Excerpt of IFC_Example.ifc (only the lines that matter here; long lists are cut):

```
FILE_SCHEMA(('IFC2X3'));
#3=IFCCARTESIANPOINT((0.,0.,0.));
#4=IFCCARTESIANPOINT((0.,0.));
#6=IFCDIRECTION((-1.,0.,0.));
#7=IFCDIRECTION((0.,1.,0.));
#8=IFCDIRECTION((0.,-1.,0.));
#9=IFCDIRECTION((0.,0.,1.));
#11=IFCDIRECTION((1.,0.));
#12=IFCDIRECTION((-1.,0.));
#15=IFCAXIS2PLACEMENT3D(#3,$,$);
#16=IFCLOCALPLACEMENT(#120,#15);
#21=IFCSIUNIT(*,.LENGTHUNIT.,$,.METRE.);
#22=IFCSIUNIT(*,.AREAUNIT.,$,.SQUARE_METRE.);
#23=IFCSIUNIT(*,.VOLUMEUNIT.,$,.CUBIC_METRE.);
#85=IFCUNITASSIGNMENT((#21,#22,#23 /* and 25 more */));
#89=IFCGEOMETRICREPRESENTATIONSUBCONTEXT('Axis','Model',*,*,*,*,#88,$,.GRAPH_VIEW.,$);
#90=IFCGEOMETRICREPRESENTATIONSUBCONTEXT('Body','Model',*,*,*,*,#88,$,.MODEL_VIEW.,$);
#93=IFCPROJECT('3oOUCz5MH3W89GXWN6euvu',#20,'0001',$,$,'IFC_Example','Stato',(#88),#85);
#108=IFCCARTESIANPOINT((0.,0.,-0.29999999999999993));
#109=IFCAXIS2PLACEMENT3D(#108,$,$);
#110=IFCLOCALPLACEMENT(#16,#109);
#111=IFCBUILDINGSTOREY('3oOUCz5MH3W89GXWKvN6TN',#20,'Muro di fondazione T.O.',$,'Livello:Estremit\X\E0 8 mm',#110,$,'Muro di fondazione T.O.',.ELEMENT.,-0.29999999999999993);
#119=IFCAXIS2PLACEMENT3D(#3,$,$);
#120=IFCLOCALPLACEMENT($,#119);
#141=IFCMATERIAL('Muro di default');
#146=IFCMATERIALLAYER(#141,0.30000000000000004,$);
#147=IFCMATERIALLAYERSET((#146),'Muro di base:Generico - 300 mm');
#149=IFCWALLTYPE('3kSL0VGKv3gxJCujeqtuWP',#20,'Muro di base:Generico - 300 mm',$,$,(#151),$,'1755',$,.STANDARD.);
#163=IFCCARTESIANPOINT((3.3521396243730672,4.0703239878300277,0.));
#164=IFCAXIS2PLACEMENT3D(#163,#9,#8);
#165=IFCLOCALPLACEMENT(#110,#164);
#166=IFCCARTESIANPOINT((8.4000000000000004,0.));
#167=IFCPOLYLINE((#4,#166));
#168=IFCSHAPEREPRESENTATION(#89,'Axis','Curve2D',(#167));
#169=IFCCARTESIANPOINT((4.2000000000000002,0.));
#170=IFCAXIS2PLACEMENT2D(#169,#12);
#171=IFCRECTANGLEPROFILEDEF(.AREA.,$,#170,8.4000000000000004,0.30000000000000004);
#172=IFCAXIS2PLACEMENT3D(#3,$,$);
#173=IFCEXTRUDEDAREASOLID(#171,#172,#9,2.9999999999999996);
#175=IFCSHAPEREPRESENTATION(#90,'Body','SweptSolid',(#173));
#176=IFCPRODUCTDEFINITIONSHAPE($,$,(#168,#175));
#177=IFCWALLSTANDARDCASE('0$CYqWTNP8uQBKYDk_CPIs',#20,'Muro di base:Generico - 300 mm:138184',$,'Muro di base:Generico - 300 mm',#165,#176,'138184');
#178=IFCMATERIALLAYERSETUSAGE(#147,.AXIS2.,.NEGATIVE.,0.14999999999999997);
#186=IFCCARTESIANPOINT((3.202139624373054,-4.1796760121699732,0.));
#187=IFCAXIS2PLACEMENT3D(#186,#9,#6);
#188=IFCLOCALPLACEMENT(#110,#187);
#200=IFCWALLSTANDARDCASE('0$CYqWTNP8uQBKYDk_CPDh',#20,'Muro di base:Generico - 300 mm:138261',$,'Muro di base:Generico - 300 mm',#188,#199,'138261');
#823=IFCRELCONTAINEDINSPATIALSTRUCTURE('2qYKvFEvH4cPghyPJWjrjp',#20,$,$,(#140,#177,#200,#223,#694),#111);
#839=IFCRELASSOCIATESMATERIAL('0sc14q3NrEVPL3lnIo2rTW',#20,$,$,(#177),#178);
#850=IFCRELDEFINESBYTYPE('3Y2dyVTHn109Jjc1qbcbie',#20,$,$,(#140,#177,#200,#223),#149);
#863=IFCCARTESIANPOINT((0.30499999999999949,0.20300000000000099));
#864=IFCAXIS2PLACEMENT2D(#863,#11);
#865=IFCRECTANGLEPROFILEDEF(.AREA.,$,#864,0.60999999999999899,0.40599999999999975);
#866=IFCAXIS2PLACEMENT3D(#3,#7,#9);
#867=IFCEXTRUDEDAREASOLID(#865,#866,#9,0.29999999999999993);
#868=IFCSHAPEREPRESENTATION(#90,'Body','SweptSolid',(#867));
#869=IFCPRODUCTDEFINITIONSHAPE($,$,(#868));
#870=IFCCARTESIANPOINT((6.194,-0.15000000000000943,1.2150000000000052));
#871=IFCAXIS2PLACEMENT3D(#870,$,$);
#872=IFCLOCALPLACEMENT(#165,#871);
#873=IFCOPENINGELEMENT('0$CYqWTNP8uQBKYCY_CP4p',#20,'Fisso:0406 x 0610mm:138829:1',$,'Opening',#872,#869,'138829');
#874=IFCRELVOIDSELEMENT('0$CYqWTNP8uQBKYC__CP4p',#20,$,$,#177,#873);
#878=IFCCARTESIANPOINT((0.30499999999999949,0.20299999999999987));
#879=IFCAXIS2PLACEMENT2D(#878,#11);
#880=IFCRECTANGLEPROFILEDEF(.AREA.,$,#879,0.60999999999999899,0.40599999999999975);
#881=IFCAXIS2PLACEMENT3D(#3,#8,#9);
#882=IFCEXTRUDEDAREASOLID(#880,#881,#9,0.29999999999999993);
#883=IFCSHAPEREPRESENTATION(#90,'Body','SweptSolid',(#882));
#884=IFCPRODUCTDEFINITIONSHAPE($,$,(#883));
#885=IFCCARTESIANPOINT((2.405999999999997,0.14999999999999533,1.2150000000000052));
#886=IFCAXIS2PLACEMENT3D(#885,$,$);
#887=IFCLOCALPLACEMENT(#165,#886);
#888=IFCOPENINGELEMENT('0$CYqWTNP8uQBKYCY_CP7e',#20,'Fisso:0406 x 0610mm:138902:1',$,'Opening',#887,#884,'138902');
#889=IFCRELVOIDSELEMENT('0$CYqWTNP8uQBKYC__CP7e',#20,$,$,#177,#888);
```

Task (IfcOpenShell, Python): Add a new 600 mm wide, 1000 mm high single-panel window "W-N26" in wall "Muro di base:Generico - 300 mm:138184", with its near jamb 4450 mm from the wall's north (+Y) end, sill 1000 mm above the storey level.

```python
import numpy as np
import ifcopenshell
import ifcopenshell.api.feature
import ifcopenshell.api.geometry
import ifcopenshell.api.root
import ifcopenshell.api.spatial
import ifcopenshell.api.type
import ifcopenshell.geom
import ifcopenshell.util.element
import ifcopenshell.util.placement
import ifcopenshell.util.representation
import ifcopenshell.util.shape
import ifcopenshell.util.unit

model = ifcopenshell.open("IFC_Example.ifc")
unit_scale = ifcopenshell.util.unit.calculate_unit_scale(model)
settings = ifcopenshell.geom.settings()


def volume(element):
    """Net volume in cubic metres, openings subtracted."""
    shape = ifcopenshell.geom.create_shape(settings, element)
    return ifcopenshell.util.shape.get_volume(shape.geometry)


wall = model.by_guid("0$CYqWTNP8uQBKYDk_CPIs")
storey = ifcopenshell.util.element.get_container(wall, ifc_class="IfcBuildingStorey")
context = ifcopenshell.util.representation.get_context(model, "Model", "Body", "MODEL_VIEW")
before = volume(wall)

width, height, from_end, sill = 0.6, 1, 4.45, 1  # metres

# The wall runs along its own X axis, and the end named is its -X end.
wall_shape = ifcopenshell.geom.create_shape(settings, wall)
x, y, z = ifcopenshell.util.shape.get_vertices(wall_shape.geometry).T
start = x.min() + from_end
face, thickness = float(y.min()), float(y.max() - y.min())
wall_matrix = ifcopenshell.util.placement.get_local_placement(wall.ObjectPlacement)
level = ifcopenshell.util.placement.get_local_placement(storey.ObjectPlacement)[2, 3]


def in_wall(x, y):
    """Placement at x, y metres in the wall's axes, at sill height."""
    matrix = wall_matrix.copy()
    matrix[:, 3] = wall_matrix @ np.array([x / unit_scale, y / unit_scale, 0.0, 1.0])
    matrix[2, 3] = level + sill / unit_scale
    return matrix


# Opening: a box that overshoots both wall faces by 50 mm.
opening = ifcopenshell.api.root.create_entity(model, ifc_class="IfcOpeningElement")
box = ifcopenshell.api.geometry.add_wall_representation(
    model, context=context, length=width, height=height, thickness=thickness + 0.1
)
ifcopenshell.api.geometry.assign_representation(model, product=opening, representation=box)
ifcopenshell.api.geometry.edit_object_placement(model, product=opening, matrix=in_wall(start, face - 0.05), is_si=False)
ifcopenshell.api.feature.add_feature(model, feature=opening, element=wall)

window = ifcopenshell.api.root.create_entity(model, ifc_class="IfcWindow", name="W-N26")
window.OverallWidth, window.OverallHeight = width / unit_scale, height / unit_scale
body = ifcopenshell.api.geometry.add_window_representation(
    model,
    context=context,
    overall_width=window.OverallWidth,
    overall_height=window.OverallHeight,
    partition_type="SINGLE_PANEL",
)
ifcopenshell.api.geometry.assign_representation(model, product=window, representation=body)
ifcopenshell.api.spatial.assign_container(model, products=[window], relating_structure=storey)
fills = ifcopenshell.api.feature.add_filling(model, opening=opening, element=window)
fills.OwnerHistory = window.OwnerHistory  # required in IFC2X3

# IFC2X3 keeps the operation on the window style.
style = ifcopenshell.api.root.create_entity(model, ifc_class="IfcWindowStyle", name="W-N26")
style.OperationType, style.ConstructionType = "SINGLE_PANEL", "NOTDEFINED"
style.ParameterTakesPrecedence = style.Sizeable = False
ifcopenshell.api.type.assign_type(model, related_objects=[window], relating_type=style)

# Centre the window in the wall's thickness.
ifcopenshell.api.geometry.edit_object_placement(model, product=window, matrix=in_wall(start, face), is_si=False)
window_shape = ifcopenshell.geom.create_shape(settings, window)
depth = ifcopenshell.util.shape.get_vertices(window_shape.geometry)[:, 1]
offset = face + thickness / 2 - (depth.min() + depth.max()) / 2
ifcopenshell.api.geometry.edit_object_placement(model, product=window, matrix=in_wall(start, offset), is_si=False)

after = volume(wall)

print(f"wall volume {before:.3f} -> {after:.3f} m3")

model.write("IFC_Example_rev.ifc")
```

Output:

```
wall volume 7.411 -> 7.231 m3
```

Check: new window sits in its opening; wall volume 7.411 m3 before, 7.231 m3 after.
